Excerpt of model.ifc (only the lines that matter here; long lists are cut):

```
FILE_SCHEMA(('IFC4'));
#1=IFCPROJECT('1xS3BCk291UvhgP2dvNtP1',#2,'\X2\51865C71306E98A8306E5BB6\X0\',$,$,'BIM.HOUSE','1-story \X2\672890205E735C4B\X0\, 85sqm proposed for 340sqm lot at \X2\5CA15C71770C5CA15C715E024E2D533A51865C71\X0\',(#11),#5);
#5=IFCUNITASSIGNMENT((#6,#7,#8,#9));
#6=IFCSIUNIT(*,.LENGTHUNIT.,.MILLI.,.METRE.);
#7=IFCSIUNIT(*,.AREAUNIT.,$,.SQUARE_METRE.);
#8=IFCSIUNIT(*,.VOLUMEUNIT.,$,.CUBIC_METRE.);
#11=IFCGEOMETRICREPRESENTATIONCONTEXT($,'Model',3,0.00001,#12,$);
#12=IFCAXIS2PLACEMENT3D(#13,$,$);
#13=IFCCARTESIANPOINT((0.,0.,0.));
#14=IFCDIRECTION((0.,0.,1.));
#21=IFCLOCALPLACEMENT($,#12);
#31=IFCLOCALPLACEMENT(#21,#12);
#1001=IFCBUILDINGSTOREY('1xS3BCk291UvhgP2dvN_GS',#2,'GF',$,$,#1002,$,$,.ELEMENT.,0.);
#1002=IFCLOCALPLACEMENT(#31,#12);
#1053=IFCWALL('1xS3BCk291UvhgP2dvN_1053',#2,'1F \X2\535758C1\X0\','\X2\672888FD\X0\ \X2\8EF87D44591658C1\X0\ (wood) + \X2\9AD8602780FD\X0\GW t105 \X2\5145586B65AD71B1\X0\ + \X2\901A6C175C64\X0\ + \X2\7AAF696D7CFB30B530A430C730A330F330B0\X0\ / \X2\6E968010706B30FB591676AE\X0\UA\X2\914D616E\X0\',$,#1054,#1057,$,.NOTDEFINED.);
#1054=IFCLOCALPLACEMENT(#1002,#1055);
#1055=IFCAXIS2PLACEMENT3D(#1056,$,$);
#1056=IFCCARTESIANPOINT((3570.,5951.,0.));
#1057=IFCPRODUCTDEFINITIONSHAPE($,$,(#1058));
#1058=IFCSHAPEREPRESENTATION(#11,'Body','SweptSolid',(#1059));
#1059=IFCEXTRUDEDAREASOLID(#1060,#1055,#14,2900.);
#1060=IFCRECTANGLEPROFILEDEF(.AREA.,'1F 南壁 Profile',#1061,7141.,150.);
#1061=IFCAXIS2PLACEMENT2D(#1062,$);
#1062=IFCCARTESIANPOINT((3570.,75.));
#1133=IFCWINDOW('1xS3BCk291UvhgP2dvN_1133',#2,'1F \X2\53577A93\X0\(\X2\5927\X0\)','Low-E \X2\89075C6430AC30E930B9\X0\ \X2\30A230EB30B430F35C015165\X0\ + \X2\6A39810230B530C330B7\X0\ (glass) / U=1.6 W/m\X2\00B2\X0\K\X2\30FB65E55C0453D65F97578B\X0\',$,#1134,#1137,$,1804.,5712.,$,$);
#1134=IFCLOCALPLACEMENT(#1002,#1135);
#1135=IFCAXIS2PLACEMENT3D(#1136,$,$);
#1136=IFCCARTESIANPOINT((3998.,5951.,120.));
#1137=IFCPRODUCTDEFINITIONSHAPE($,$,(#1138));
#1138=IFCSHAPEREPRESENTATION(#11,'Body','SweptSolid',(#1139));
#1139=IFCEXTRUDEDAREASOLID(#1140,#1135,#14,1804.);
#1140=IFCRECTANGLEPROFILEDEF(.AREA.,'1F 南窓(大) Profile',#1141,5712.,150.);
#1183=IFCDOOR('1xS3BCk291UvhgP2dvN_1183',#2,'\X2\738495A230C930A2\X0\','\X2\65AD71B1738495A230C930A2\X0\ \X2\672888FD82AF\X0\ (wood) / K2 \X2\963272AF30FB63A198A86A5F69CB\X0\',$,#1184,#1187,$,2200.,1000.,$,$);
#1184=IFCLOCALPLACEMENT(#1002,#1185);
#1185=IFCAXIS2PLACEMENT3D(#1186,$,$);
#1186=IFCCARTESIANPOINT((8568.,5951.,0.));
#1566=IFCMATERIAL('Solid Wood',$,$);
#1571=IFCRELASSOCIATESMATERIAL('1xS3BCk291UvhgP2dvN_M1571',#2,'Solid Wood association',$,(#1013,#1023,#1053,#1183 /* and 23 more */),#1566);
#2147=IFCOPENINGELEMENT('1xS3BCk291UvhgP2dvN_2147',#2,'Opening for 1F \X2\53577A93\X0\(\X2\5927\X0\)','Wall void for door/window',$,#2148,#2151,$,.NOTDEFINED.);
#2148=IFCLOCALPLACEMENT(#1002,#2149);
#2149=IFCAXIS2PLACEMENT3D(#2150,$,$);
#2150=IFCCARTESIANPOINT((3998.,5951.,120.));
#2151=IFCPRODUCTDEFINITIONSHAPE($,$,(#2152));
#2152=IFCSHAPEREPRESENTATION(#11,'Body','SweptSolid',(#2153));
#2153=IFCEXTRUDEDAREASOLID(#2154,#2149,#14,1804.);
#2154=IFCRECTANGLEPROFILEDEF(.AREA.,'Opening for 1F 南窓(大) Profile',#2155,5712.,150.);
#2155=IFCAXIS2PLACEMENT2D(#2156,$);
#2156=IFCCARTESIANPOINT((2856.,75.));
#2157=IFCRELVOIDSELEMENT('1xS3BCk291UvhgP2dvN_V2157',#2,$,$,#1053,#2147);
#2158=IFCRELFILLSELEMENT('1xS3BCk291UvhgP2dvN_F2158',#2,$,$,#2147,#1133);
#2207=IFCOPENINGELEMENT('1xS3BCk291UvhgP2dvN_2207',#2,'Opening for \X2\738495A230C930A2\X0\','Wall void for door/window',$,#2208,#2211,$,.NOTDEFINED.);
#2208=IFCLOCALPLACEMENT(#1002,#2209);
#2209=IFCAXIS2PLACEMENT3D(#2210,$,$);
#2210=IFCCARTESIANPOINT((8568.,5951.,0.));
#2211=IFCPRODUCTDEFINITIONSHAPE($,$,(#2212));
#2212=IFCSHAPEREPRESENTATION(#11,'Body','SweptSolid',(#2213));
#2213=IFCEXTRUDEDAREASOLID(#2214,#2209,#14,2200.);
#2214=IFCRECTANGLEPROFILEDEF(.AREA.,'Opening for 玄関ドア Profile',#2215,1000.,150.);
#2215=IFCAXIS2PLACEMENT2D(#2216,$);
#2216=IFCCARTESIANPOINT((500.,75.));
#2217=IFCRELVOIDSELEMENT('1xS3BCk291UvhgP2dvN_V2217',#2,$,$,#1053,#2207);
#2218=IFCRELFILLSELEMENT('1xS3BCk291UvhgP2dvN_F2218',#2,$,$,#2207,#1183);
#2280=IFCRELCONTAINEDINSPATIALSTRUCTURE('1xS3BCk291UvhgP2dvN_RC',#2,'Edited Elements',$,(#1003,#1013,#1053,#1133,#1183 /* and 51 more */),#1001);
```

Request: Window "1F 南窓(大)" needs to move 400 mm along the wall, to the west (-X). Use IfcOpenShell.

```python
import ifcopenshell
import ifcopenshell.api.geometry
import ifcopenshell.util.placement
import ifcopenshell.util.unit

model = ifcopenshell.open("model.ifc")
unit_scale = ifcopenshell.util.unit.calculate_unit_scale(model)

window = model.by_id(1133)
opening = window.FillsVoids[0].RelatingOpeningElement
wall = opening.VoidsElements[0].RelatingBuildingElement

wall_matrix = ifcopenshell.util.placement.get_local_placement(wall.ObjectPlacement)
shift = wall_matrix[:3, 0] * -0.4 / unit_scale
before = ifcopenshell.util.placement.get_local_placement(window.ObjectPlacement)[:3, 3].copy()

# The window is not placed relative to its opening, so move both.
for product in (opening, window):
    matrix = ifcopenshell.util.placement.get_local_placement(product.ObjectPlacement)
    matrix[:3, 3] += shift
    ifcopenshell.api.geometry.edit_object_placement(model, product=product, matrix=matrix, is_si=False)

after = ifcopenshell.util.placement.get_local_placement(window.ObjectPlacement)[:3, 3]
print("window moved by", (after - before).round(3) + 0.0)

model.write("model_rev.ifc")
```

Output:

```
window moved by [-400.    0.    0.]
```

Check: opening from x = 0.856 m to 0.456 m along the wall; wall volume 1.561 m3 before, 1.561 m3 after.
